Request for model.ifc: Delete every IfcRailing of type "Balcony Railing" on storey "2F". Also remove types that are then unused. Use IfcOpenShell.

First a look at what the model holds.

```python
import ifcopenshell
import ifcopenshell.util.element

model = ifcopenshell.open("model.ifc")
print(model.schema)
storey = next(s for s in model.by_type("IfcBuildingStorey") if s.Name == "2F")
railings = [e for e in ifcopenshell.util.element.get_decomposition(storey) if e.is_a("IfcRailing")]
seen = {}
for e in railings:
    element_type = ifcopenshell.util.element.get_type(e)
    name = element_type.Name if element_type not in (None, e) else None
    seen[name] = seen.get(name, 0) + 1
for name, count in sorted(seen.items(), key=str):
    print(count, "x", name)
```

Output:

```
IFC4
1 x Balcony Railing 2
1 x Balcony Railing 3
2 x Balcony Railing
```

```python
import ifcopenshell
import ifcopenshell.api.root
import ifcopenshell.util.element

model = ifcopenshell.open("model.ifc")

storey = next(s for s in model.by_type("IfcBuildingStorey") if s.Name == "2F")
railings = [e for e in ifcopenshell.util.element.get_decomposition(storey) if e.is_a("IfcRailing")]
targets = [e for e in railings if (t := ifcopenshell.util.element.get_type(e)) not in (None, e) and t.Name == "Balcony Railing"]
types = {ifcopenshell.util.element.get_type(e) for e in targets} - {None, *targets}

for e in targets:
    ifcopenshell.api.root.remove_product(model, product=e)
print(len(targets), "removed")

unused = [t for t in types if not ifcopenshell.util.element.get_types(t)]
for t in unused:
    ifcopenshell.api.root.remove_product(model, product=t)
print(len(unused), "unused types removed")

model.write("model_updated.ifc")
```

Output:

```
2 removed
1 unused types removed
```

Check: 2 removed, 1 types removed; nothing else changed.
